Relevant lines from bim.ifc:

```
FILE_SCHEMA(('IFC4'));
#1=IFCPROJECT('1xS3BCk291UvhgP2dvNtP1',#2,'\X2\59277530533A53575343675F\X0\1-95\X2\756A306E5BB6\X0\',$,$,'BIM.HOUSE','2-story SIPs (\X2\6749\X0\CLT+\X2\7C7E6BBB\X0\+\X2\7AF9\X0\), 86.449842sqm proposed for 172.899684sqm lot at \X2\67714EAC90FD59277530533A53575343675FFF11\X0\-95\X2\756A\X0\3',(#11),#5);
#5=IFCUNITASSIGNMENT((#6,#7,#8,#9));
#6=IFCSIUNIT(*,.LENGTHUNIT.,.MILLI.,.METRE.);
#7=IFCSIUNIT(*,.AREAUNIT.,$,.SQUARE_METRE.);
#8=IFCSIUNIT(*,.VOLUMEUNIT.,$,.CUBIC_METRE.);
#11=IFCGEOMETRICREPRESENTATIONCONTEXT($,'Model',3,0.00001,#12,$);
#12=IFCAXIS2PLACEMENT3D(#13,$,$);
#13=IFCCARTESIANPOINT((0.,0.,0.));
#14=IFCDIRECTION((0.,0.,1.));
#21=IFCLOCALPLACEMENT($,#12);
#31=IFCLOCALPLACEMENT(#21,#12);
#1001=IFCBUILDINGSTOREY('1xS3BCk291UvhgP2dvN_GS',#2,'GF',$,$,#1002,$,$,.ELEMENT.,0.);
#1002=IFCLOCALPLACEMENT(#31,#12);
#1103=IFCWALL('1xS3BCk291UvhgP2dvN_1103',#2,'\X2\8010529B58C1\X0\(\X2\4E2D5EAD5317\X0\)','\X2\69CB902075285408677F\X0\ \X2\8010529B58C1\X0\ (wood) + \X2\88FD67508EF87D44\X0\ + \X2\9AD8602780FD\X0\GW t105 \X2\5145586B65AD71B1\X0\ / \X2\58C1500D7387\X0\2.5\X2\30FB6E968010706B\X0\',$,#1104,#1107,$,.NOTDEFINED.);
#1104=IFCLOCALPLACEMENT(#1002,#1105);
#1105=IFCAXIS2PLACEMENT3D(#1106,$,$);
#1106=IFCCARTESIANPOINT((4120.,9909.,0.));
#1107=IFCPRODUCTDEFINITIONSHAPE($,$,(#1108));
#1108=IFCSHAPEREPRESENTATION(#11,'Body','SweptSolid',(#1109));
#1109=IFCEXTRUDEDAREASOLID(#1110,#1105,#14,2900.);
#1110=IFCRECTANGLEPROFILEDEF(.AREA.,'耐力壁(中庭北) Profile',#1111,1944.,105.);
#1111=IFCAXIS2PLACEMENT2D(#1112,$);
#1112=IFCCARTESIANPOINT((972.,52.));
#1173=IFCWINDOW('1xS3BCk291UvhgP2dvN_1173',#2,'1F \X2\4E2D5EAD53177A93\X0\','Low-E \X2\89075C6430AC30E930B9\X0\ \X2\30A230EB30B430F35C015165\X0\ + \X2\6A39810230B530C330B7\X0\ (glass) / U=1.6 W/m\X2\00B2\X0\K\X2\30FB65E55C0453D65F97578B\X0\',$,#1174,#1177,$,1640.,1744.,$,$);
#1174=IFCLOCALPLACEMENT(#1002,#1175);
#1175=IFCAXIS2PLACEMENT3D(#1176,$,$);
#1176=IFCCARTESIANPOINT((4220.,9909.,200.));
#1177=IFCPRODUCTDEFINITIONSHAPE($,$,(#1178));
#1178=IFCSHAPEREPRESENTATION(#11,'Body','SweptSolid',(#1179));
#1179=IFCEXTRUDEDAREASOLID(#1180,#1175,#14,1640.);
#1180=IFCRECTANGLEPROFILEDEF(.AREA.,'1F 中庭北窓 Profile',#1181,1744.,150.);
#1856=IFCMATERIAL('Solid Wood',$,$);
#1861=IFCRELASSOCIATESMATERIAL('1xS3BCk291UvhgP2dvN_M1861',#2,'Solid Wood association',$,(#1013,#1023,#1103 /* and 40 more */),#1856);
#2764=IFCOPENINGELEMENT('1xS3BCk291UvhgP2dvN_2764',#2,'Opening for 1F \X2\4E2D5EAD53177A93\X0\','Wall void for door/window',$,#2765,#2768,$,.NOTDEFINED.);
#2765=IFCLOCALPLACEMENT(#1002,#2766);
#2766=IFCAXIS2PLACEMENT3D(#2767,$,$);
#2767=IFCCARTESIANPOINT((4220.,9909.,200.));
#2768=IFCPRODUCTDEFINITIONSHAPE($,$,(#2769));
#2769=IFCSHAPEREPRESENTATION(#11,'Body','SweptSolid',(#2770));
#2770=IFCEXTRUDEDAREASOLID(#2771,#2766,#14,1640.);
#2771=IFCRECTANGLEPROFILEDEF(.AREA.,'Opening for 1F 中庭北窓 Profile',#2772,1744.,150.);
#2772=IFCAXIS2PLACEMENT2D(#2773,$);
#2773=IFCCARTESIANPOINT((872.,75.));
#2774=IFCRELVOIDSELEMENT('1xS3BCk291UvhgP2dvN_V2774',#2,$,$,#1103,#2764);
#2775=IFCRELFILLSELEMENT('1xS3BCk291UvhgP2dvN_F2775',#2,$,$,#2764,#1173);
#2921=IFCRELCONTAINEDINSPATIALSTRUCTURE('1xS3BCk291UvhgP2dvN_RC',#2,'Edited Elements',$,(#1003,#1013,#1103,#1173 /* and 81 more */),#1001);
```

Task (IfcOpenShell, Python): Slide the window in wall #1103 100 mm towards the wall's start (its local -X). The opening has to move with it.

```python
import ifcopenshell
import ifcopenshell.api.geometry
import ifcopenshell.util.placement
import ifcopenshell.util.unit

model = ifcopenshell.open("bim.ifc")
unit_scale = ifcopenshell.util.unit.calculate_unit_scale(model)

window = model.by_guid("1xS3BCk291UvhgP2dvN_1173")
opening = window.FillsVoids[0].RelatingOpeningElement
wall = opening.VoidsElements[0].RelatingBuildingElement

wall_matrix = ifcopenshell.util.placement.get_local_placement(wall.ObjectPlacement)
shift = wall_matrix[:3, 0] * -0.1 / unit_scale
before = ifcopenshell.util.placement.get_local_placement(window.ObjectPlacement)[:3, 3].copy()

# The window is not placed relative to its opening, so move both.
for product in (opening, window):
    matrix = ifcopenshell.util.placement.get_local_placement(product.ObjectPlacement)
    matrix[:3, 3] += shift
    ifcopenshell.api.geometry.edit_object_placement(model, product=product, matrix=matrix, is_si=False)

after = ifcopenshell.util.placement.get_local_placement(window.ObjectPlacement)[:3, 3]
print("window moved by", (after - before).round(3) + 0.0)

model.write("bim_edited.ifc")
```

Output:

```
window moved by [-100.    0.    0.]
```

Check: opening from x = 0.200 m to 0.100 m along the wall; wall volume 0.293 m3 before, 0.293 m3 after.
